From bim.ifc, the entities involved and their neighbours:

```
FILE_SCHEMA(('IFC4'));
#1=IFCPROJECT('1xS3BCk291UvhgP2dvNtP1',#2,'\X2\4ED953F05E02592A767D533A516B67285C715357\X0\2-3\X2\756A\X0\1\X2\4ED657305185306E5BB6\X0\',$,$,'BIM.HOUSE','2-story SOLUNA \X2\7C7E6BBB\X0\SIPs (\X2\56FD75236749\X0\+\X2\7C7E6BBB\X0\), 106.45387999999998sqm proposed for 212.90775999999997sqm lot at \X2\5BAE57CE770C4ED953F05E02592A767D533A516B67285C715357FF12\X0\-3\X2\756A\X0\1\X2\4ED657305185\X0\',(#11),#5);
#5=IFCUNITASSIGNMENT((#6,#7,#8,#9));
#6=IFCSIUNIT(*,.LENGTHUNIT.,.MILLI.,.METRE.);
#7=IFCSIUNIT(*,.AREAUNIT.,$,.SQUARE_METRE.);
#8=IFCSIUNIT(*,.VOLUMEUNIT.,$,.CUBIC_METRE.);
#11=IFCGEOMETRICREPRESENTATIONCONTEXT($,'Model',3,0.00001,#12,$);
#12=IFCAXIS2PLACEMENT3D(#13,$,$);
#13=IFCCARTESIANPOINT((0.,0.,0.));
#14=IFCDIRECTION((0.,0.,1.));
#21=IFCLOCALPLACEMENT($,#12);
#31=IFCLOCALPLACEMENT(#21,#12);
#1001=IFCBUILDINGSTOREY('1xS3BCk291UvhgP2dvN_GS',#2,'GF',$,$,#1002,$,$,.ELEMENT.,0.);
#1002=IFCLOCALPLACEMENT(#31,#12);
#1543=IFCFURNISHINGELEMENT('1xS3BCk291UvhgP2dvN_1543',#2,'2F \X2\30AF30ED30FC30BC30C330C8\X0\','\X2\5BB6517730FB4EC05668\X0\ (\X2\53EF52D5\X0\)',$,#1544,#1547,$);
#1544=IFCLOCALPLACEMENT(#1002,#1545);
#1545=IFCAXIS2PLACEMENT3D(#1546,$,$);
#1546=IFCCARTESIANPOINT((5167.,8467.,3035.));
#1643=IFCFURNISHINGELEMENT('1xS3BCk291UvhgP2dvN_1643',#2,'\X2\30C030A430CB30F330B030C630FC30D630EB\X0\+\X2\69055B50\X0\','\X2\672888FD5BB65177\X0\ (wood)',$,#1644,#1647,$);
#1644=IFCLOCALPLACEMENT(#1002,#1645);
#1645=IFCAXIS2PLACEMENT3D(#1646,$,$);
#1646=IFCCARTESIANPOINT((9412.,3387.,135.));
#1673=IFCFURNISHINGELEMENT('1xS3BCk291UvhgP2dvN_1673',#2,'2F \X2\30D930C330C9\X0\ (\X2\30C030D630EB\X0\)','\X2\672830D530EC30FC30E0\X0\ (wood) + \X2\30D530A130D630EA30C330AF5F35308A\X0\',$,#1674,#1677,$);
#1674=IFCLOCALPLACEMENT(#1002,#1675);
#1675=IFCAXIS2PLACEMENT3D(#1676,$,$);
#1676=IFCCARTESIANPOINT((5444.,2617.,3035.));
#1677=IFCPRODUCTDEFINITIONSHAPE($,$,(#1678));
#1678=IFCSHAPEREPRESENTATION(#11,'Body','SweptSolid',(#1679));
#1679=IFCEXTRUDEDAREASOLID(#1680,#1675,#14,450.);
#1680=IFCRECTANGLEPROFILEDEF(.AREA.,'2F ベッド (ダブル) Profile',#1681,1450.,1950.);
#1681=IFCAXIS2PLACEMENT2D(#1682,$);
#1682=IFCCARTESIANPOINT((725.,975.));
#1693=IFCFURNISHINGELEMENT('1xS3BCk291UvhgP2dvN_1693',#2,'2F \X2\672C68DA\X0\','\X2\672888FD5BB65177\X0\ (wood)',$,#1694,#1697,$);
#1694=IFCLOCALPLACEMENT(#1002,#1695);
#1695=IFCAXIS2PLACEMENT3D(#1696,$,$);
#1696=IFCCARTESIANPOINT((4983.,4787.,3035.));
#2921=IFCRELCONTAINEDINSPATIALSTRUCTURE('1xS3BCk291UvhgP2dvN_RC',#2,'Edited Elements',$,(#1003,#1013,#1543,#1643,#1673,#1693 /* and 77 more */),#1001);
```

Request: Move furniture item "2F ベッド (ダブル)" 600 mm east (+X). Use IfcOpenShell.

```python
import ifcopenshell
import ifcopenshell.api.geometry
import ifcopenshell.util.placement

model = ifcopenshell.open("bim.ifc")

item = model.by_guid("1xS3BCk291UvhgP2dvN_1673")
matrix = ifcopenshell.util.placement.get_local_placement(item.ObjectPlacement)
matrix[0, 3] += 600.0
ifcopenshell.api.geometry.edit_object_placement(model, product=item, matrix=matrix, is_si=False)

print(ifcopenshell.util.placement.get_local_placement(item.ObjectPlacement).round(3) + 0.0)

model.write("bim_edited.ifc")
```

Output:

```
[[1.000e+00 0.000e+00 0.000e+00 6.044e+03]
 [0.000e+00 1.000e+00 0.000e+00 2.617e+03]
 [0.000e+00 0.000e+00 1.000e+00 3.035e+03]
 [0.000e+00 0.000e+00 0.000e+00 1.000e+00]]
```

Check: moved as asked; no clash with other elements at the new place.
